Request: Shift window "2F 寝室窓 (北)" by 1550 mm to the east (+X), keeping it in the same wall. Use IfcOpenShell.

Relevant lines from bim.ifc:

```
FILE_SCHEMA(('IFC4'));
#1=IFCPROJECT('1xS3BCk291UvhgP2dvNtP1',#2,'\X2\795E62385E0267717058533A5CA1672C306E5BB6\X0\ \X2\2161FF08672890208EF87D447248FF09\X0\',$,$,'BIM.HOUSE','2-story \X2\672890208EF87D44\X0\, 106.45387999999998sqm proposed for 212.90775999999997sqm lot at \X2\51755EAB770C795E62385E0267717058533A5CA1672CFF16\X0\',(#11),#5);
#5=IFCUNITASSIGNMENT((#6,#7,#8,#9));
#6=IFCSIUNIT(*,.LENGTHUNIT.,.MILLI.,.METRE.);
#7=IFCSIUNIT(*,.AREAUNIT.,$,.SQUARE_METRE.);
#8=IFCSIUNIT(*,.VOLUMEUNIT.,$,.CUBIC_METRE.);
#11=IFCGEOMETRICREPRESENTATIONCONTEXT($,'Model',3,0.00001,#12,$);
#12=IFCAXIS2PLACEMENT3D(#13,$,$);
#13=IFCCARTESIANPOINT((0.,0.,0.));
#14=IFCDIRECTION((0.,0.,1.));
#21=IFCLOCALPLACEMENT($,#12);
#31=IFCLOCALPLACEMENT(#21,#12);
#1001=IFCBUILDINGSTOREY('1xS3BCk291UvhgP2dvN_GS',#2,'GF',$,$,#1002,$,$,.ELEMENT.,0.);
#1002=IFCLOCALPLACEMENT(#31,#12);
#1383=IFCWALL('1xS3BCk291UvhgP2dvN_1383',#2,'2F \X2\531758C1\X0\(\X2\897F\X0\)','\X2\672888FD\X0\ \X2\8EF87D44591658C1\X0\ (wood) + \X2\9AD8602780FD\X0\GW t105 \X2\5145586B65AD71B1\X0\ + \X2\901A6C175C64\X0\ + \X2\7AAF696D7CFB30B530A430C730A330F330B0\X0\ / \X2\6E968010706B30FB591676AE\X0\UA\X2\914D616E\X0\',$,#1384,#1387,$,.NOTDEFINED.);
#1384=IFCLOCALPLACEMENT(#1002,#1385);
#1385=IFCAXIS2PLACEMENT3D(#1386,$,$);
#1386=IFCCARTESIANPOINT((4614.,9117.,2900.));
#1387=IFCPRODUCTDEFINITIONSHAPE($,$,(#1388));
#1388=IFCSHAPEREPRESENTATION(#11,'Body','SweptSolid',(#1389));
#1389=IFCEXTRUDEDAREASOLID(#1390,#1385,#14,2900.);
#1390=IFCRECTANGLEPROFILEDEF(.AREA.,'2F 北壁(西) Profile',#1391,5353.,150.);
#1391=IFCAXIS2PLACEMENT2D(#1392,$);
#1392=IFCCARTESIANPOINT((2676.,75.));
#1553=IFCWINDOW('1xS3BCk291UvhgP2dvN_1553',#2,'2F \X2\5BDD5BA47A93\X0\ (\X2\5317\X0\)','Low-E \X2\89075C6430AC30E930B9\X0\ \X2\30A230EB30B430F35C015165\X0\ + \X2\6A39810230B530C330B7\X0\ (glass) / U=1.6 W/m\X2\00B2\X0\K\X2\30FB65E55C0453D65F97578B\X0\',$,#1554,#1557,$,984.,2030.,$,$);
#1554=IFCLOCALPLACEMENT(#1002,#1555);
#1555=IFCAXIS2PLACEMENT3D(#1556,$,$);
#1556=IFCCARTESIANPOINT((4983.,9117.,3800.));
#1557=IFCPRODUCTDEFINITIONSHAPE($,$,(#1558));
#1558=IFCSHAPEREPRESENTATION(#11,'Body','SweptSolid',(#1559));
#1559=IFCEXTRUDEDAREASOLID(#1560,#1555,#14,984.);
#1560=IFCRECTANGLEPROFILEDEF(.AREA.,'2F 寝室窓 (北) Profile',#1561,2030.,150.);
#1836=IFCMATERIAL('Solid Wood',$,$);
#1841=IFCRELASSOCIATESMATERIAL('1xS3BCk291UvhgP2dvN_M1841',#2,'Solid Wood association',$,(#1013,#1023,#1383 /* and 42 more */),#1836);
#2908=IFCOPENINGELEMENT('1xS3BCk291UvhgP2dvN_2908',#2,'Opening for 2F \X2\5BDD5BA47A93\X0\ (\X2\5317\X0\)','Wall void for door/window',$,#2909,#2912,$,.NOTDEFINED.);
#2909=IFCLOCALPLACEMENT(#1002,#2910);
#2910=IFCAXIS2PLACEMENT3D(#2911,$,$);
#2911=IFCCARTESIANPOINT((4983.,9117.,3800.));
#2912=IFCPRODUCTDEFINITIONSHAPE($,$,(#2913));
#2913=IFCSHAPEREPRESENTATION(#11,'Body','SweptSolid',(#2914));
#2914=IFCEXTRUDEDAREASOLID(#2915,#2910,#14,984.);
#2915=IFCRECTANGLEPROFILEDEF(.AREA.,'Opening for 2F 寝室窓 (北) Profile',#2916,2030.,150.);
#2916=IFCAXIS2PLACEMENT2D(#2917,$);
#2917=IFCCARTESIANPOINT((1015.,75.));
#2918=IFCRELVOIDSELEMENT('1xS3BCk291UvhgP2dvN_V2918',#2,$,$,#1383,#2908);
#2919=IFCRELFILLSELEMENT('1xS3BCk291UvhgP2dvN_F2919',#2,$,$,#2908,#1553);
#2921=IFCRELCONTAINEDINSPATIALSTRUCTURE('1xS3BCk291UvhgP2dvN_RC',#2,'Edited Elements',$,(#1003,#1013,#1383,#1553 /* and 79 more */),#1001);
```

```python
import ifcopenshell
import ifcopenshell.api.geometry
import ifcopenshell.util.placement

model = ifcopenshell.open("bim.ifc")

window = model.by_guid("1xS3BCk291UvhgP2dvN_1553")
opening = window.FillsVoids[0].RelatingOpeningElement
wall = opening.VoidsElements[0].RelatingBuildingElement

wall_matrix = ifcopenshell.util.placement.get_local_placement(wall.ObjectPlacement)
shift = wall_matrix[:3, 0] * 1550.0
before = ifcopenshell.util.placement.get_local_placement(window.ObjectPlacement)[:3, 3].copy()

# The window is not placed relative to its opening, so move both.
for product in (opening, window):
    matrix = ifcopenshell.util.placement.get_local_placement(product.ObjectPlacement)
    matrix[:3, 3] += shift
    ifcopenshell.api.geometry.edit_object_placement(model, product=product, matrix=matrix, is_si=False)

after = ifcopenshell.util.placement.get_local_placement(window.ObjectPlacement)[:3, 3]
print("window moved by", (after - before).round(3) + 0.0)

model.write("bim_rev.ifc")
```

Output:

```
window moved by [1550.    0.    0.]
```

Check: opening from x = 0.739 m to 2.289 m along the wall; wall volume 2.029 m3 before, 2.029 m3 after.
